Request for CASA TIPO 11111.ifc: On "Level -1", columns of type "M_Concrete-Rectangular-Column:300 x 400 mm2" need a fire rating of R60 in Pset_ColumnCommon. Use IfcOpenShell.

First a look at what the model holds.

```python
import ifcopenshell
import ifcopenshell.util.element

model = ifcopenshell.open("CASA TIPO 11111.ifc")
print(model.schema)
storey = next(s for s in model.by_type("IfcBuildingStorey") if s.Name == "Level -1")
columns = [e for e in ifcopenshell.util.element.get_decomposition(storey) if e.is_a("IfcColumn")]
seen = {}
for e in columns:
    element_type = ifcopenshell.util.element.get_type(e)
    key = (element_type.Name if element_type != e and element_type else None, ifcopenshell.util.element.get_pset(e, "Pset_ColumnCommon", "FireRating"))
    seen[key] = seen.get(key, 0) + 1
for (name, value), count in sorted(seen.items(), key=str):
    print(count, "x", name, "|", value)
```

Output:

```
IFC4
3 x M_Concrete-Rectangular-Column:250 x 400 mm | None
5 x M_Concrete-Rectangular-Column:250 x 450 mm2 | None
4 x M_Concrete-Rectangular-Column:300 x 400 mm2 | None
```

```python
import ifcopenshell
import ifcopenshell.api.pset
import ifcopenshell.util.element

model = ifcopenshell.open("CASA TIPO 11111.ifc")

storey = next(s for s in model.by_type("IfcBuildingStorey") if s.Name == "Level -1")
columns = [e for e in ifcopenshell.util.element.get_decomposition(storey) if e.is_a("IfcColumn")]

count = 0
for e in columns:
    element_type = ifcopenshell.util.element.get_type(e)
    if element_type in (None, e) or element_type.Name != "M_Concrete-Rectangular-Column:300 x 400 mm2":
        continue
    # add_pset returns the element's existing set when there is one.
    pset = ifcopenshell.api.pset.add_pset(model, product=e, name="Pset_ColumnCommon")
    ifcopenshell.api.pset.edit_pset(model, pset=pset, properties={"FireRating": "R60"})
    count += 1

print(count, "columns updated")

model.write("CASA TIPO 11111_updated.ifc")
```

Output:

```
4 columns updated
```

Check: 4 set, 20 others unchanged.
